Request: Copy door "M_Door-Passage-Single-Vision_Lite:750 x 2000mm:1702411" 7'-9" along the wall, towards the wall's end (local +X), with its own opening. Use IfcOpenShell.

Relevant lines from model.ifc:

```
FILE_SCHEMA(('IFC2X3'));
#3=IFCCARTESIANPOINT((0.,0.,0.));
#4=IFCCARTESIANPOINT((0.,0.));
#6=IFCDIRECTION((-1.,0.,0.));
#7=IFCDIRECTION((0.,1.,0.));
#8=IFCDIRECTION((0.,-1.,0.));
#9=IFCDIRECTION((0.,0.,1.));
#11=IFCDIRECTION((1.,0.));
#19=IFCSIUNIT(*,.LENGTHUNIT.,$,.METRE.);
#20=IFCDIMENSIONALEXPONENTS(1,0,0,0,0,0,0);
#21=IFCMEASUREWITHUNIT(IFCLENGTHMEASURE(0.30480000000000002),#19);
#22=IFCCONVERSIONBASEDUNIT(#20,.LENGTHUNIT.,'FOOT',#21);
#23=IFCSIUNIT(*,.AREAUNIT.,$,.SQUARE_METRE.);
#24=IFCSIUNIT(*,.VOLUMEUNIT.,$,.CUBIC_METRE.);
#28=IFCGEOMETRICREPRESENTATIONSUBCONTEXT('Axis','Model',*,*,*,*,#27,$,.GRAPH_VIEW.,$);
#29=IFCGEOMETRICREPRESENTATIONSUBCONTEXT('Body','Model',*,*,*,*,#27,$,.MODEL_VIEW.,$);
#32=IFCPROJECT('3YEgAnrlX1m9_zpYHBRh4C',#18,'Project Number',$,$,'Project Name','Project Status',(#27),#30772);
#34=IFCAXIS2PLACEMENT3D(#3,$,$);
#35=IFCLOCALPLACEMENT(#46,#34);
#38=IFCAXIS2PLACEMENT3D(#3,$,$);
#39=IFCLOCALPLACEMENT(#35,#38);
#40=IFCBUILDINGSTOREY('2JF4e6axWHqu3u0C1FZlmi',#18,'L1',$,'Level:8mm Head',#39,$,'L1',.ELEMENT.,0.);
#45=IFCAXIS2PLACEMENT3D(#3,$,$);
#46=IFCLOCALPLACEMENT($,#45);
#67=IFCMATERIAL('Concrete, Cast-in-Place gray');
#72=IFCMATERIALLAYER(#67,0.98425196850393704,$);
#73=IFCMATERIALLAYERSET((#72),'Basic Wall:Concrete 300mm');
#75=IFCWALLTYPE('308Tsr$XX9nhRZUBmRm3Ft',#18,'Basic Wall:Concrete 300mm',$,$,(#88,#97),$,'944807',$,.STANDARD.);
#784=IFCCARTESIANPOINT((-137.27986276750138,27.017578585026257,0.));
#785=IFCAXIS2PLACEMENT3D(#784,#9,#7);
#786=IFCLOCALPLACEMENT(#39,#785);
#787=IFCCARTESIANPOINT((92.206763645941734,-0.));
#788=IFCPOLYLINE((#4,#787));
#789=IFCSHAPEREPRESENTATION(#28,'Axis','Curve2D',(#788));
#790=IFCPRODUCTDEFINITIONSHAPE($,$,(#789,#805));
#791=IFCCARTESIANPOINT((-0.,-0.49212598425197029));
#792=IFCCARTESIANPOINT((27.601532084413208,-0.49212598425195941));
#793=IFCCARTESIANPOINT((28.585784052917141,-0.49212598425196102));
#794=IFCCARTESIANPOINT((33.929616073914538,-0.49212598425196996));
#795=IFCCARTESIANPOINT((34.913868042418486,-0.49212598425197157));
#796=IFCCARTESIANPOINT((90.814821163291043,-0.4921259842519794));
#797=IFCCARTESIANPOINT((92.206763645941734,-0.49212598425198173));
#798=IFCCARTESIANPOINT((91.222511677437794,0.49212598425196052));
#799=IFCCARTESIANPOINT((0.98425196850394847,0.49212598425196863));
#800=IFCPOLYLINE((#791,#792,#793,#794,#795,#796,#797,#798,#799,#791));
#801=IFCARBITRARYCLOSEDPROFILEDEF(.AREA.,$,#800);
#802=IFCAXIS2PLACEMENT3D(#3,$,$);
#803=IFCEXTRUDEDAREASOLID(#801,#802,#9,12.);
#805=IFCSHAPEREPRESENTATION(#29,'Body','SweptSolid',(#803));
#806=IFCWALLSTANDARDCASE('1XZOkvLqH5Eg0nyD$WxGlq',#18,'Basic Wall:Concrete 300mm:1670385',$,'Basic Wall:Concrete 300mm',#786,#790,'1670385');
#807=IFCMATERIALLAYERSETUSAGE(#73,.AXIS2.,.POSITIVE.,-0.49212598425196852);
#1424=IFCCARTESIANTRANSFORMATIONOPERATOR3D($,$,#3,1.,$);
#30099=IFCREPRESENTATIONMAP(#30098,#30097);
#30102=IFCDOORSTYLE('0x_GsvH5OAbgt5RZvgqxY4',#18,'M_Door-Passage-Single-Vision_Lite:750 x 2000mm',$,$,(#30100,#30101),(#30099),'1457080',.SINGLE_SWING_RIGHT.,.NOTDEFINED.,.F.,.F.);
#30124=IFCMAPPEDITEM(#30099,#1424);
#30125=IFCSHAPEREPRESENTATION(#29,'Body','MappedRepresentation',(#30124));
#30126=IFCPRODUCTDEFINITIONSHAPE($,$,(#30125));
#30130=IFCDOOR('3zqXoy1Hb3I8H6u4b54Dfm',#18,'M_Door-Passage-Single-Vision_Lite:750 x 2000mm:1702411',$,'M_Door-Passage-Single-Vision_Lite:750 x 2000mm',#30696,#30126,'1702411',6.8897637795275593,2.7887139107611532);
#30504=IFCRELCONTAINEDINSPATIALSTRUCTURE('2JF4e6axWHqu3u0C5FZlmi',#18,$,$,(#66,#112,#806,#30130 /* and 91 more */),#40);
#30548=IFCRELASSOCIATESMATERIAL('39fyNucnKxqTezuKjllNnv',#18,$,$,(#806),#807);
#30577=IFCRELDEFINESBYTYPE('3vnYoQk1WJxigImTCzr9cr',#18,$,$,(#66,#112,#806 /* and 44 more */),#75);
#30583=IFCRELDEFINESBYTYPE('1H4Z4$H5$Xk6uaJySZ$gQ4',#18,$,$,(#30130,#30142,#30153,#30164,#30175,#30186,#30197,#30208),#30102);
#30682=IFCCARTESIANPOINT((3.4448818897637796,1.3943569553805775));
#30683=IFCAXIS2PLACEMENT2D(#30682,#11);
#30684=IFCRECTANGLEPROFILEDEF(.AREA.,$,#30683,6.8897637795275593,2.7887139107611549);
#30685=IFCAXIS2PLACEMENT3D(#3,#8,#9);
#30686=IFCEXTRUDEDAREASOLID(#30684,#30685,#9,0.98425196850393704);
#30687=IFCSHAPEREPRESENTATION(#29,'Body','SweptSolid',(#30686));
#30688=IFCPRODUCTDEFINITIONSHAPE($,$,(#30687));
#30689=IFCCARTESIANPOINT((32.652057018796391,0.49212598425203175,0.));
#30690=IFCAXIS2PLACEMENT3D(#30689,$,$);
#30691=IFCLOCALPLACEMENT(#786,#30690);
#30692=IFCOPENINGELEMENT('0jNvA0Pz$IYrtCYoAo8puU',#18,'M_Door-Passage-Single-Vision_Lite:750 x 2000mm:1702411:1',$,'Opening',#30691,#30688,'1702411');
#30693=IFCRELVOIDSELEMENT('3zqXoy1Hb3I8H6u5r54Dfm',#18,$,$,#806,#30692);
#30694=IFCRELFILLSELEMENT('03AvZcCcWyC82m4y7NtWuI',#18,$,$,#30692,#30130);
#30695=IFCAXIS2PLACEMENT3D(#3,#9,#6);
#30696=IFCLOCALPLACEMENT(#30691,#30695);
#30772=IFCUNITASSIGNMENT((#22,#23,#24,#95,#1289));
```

```python
import ifcopenshell
import ifcopenshell.api.feature
import ifcopenshell.api.geometry
import ifcopenshell.api.root
import ifcopenshell.geom
import ifcopenshell.util.element
import ifcopenshell.util.placement
import ifcopenshell.util.shape
import ifcopenshell.util.unit

model = ifcopenshell.open("model.ifc")
unit_scale = ifcopenshell.util.unit.calculate_unit_scale(model)
settings = ifcopenshell.geom.settings()


def volume(element):
    """Net volume in cubic metres, openings subtracted."""
    shape = ifcopenshell.geom.create_shape(settings, element)
    return ifcopenshell.util.shape.get_volume(shape.geometry)


def reuse_history(source, copy):
    """copy_class also copies each property set's owner history, people and application; keep the originals."""
    for rel in copy.IsDefinedBy:
        if rel.is_a("IfcRelDefinesByProperties") and (history := rel.RelatingPropertyDefinition.OwnerHistory):
            rel.RelatingPropertyDefinition.OwnerHistory = source.OwnerHistory
            ifcopenshell.util.element.remove_deep2(model, history)


door = model.by_guid("3zqXoy1Hb3I8H6u4b54Dfm")
opening = door.FillsVoids[0].RelatingOpeningElement
wall = opening.VoidsElements[0].RelatingBuildingElement
before = volume(wall)
shift = ifcopenshell.util.placement.get_local_placement(wall.ObjectPlacement)[:3, 0] * 93 * 0.0254 / unit_scale

# copy_class copies the void relationship, type, container and properties, but no geometry.
new_opening = ifcopenshell.api.root.copy_class(model, product=opening)
new_opening.Representation = ifcopenshell.util.element.copy_deep(
    model, opening.Representation, exclude=["IfcGeometricRepresentationContext", "IfcRepresentationMap"]
)
new_opening.Name = "M_Door-Passage-Single-Vision_Lite:750 x 2000mm"
new_opening.Tag = None
new_door = ifcopenshell.api.root.copy_class(model, product=door)
new_door.Representation = ifcopenshell.util.element.copy_deep(
    model, door.Representation, exclude=["IfcGeometricRepresentationContext", "IfcRepresentationMap"]
)
new_door.Name = "M_Door-Passage-Single-Vision_Lite:750 x 2000mm"
new_door.Tag = None
reuse_history(door, new_door)
fills = ifcopenshell.api.feature.add_filling(model, opening=new_opening, element=new_door)
fills.OwnerHistory = new_door.OwnerHistory  # required in IFC2X3

for old, new in ((opening, new_opening), (door, new_door)):
    matrix = ifcopenshell.util.placement.get_local_placement(old.ObjectPlacement)
    matrix[:3, 3] += shift
    ifcopenshell.api.geometry.edit_object_placement(model, product=new, matrix=matrix, is_si=False)

after = volume(wall)

print(f"wall volume {before:.3f} -> {after:.3f} m3")

model.write("model_updated.ifc")
```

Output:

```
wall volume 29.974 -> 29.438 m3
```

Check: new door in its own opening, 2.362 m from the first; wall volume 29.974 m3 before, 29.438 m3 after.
